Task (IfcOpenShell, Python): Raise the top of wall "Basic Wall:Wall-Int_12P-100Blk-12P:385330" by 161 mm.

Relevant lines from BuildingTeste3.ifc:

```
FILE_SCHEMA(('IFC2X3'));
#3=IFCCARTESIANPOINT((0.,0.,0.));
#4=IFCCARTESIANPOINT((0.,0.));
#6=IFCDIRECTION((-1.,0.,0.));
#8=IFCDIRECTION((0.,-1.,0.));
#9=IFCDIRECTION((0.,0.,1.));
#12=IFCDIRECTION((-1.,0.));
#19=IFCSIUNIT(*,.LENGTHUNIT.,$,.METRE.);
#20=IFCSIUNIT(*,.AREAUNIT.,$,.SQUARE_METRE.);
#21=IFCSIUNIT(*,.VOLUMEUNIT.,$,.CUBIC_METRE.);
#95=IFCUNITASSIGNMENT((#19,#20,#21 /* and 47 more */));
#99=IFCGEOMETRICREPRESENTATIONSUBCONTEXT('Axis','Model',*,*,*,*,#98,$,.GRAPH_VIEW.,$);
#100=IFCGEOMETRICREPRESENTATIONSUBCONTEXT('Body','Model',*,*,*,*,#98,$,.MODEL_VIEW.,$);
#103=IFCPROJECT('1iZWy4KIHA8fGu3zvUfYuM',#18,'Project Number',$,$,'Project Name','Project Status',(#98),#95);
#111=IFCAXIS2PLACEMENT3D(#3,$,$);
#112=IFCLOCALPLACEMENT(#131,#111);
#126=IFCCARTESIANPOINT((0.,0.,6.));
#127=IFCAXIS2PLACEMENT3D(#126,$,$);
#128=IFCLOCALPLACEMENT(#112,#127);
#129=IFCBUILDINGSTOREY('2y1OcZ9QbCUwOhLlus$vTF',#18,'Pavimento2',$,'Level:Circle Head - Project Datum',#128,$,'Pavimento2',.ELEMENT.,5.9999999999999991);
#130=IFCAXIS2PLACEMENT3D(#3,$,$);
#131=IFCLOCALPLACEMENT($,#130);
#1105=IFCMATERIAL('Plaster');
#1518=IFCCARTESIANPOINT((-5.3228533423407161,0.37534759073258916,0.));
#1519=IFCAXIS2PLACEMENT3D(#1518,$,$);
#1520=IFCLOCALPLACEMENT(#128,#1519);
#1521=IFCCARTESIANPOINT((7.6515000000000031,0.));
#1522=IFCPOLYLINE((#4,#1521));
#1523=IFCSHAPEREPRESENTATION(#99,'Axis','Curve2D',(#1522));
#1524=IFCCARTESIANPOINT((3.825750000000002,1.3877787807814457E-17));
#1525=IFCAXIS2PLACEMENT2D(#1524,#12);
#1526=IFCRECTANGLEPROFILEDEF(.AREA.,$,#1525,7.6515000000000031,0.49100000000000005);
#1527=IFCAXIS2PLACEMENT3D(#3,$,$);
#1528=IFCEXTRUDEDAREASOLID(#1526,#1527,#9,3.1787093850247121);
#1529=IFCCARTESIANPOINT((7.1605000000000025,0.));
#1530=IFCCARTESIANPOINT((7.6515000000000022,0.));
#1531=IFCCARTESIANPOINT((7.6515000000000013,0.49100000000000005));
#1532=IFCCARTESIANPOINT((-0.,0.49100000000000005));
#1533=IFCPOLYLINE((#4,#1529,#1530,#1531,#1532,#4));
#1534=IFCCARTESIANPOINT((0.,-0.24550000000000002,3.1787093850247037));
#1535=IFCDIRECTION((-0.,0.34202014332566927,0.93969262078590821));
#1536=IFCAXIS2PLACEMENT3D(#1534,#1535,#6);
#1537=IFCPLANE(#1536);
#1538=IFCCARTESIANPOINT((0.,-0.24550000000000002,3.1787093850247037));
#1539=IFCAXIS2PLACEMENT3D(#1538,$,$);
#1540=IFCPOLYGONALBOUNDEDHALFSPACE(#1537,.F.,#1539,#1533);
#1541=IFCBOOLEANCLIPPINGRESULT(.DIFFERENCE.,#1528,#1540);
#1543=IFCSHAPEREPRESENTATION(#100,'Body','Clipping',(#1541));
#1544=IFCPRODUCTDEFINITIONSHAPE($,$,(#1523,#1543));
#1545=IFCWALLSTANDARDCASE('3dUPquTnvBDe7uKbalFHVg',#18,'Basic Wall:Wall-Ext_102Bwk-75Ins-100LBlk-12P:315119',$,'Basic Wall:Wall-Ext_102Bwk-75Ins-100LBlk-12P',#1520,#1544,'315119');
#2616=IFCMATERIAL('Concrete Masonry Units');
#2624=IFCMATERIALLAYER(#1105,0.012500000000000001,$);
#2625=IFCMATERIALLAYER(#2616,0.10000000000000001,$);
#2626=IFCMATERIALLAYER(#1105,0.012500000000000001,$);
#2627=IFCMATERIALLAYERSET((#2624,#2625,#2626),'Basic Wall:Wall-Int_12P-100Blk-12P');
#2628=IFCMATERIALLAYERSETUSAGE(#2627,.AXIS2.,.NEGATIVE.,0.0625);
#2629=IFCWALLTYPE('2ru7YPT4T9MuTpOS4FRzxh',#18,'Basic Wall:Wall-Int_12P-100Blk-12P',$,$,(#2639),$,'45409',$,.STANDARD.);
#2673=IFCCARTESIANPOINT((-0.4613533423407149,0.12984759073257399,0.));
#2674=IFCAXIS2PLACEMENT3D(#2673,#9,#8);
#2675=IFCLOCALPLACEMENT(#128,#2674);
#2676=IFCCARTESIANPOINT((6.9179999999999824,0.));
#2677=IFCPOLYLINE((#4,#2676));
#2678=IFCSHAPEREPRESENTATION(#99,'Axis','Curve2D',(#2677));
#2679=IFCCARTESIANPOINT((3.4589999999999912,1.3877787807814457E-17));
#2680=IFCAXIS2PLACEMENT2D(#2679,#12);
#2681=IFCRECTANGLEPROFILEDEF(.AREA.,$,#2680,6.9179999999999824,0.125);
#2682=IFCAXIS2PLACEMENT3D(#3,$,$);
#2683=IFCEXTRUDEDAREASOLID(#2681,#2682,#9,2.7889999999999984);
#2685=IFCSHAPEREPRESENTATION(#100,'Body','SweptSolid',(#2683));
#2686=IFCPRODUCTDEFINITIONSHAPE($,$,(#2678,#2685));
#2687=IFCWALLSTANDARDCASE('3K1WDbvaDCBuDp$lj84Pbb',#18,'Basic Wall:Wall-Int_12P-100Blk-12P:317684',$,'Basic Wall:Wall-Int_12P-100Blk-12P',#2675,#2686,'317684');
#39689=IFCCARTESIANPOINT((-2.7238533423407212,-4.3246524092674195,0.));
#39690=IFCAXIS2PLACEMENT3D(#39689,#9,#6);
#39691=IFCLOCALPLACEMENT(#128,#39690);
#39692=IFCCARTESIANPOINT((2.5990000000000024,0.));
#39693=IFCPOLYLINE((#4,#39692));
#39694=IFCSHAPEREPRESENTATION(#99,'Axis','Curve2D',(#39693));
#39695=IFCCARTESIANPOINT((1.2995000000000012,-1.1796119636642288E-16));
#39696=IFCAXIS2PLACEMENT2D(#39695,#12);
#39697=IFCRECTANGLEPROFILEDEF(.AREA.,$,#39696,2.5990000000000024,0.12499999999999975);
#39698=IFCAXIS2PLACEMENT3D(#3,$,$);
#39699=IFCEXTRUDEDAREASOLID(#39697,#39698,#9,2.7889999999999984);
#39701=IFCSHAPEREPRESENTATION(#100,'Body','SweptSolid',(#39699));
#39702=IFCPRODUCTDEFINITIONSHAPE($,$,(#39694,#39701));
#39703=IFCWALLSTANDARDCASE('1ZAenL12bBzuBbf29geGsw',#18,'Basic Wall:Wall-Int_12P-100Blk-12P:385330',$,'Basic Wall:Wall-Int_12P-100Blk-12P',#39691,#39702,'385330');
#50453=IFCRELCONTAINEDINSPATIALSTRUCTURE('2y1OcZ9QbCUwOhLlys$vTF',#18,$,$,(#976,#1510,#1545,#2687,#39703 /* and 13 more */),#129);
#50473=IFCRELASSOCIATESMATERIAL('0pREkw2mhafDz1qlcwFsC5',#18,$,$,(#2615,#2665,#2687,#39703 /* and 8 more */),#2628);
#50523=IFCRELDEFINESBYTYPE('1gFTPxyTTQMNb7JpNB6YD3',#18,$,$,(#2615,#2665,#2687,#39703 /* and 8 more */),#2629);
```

```python
import ifcopenshell
import ifcopenshell.geom
import ifcopenshell.util.representation
import ifcopenshell.util.shape
import ifcopenshell.util.unit

model = ifcopenshell.open("BuildingTeste3.ifc")
unit_scale = ifcopenshell.util.unit.calculate_unit_scale(model)
settings = ifcopenshell.geom.settings()


def volume(element):
    """Net volume in cubic metres, openings subtracted."""
    shape = ifcopenshell.geom.create_shape(settings, element)
    return ifcopenshell.util.shape.get_volume(shape.geometry)


wall = model.by_guid("1ZAenL12bBzuBbf29geGsw")
before = volume(wall)

body = ifcopenshell.util.representation.get_representation(wall, "Model", "Body")
solid = body.Items[0]
old_height = solid.Depth
solid.Depth += 0.161 / unit_scale
after = volume(wall)

print(f"height {old_height:g} -> {solid.Depth:g}, volume {before:.3f} -> {after:.3f} m3")

model.write("BuildingTeste3-out.ifc")
```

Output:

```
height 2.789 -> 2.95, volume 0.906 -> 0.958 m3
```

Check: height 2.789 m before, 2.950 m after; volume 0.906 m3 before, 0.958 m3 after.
